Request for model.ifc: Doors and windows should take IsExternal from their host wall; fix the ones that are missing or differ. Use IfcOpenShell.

First a look at what the model holds.

```python
import ifcopenshell
import ifcopenshell.util.element

model = ifcopenshell.open("model.ifc")
print(model.schema)
seen = {}
for e in model.by_type("IfcDoor") + model.by_type("IfcWindow"):
    if not e.FillsVoids:
        continue
    host = e.FillsVoids[0].RelatingOpeningElement.VoidsElements[0].RelatingBuildingElement
    own = ifcopenshell.util.element.get_pset(e, f"Pset_{e.is_a()[3:].removesuffix('StandardCase')}Common", "IsExternal")
    wall = ifcopenshell.util.element.get_pset(host, "Pset_WallCommon", "IsExternal")
    seen[e.is_a(), own, wall] = seen.get((e.is_a(), own, wall), 0) + 1
for (cls, own, wall), count in sorted(seen.items(), key=str):
    print(count, cls, "IsExternal:", own, "| host wall:", wall)
```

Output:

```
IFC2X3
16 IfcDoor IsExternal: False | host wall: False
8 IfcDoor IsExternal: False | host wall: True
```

```python
import ifcopenshell
import ifcopenshell.api.pset
import ifcopenshell.util.element

model = ifcopenshell.open("model.ifc")

count = 0
for ifc_class, pset_name in (("IfcDoor", "Pset_DoorCommon"), ("IfcWindow", "Pset_WindowCommon")):
    for e in model.by_type(ifc_class):
        if not e.FillsVoids:
            continue
        host = e.FillsVoids[0].RelatingOpeningElement.VoidsElements[0].RelatingBuildingElement
        external = ifcopenshell.util.element.get_pset(host, "Pset_WallCommon", "IsExternal")
        if external is None or ifcopenshell.util.element.get_pset(e, pset_name, "IsExternal") == external:
            continue
        pset = ifcopenshell.api.pset.add_pset(model, product=e, name=pset_name)
        ifcopenshell.api.pset.edit_pset(model, pset=pset, properties={"IsExternal": external})
        count += 1

print(count, "updated")

model.write("model_updated.ifc")
```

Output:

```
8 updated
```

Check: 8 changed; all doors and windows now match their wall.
